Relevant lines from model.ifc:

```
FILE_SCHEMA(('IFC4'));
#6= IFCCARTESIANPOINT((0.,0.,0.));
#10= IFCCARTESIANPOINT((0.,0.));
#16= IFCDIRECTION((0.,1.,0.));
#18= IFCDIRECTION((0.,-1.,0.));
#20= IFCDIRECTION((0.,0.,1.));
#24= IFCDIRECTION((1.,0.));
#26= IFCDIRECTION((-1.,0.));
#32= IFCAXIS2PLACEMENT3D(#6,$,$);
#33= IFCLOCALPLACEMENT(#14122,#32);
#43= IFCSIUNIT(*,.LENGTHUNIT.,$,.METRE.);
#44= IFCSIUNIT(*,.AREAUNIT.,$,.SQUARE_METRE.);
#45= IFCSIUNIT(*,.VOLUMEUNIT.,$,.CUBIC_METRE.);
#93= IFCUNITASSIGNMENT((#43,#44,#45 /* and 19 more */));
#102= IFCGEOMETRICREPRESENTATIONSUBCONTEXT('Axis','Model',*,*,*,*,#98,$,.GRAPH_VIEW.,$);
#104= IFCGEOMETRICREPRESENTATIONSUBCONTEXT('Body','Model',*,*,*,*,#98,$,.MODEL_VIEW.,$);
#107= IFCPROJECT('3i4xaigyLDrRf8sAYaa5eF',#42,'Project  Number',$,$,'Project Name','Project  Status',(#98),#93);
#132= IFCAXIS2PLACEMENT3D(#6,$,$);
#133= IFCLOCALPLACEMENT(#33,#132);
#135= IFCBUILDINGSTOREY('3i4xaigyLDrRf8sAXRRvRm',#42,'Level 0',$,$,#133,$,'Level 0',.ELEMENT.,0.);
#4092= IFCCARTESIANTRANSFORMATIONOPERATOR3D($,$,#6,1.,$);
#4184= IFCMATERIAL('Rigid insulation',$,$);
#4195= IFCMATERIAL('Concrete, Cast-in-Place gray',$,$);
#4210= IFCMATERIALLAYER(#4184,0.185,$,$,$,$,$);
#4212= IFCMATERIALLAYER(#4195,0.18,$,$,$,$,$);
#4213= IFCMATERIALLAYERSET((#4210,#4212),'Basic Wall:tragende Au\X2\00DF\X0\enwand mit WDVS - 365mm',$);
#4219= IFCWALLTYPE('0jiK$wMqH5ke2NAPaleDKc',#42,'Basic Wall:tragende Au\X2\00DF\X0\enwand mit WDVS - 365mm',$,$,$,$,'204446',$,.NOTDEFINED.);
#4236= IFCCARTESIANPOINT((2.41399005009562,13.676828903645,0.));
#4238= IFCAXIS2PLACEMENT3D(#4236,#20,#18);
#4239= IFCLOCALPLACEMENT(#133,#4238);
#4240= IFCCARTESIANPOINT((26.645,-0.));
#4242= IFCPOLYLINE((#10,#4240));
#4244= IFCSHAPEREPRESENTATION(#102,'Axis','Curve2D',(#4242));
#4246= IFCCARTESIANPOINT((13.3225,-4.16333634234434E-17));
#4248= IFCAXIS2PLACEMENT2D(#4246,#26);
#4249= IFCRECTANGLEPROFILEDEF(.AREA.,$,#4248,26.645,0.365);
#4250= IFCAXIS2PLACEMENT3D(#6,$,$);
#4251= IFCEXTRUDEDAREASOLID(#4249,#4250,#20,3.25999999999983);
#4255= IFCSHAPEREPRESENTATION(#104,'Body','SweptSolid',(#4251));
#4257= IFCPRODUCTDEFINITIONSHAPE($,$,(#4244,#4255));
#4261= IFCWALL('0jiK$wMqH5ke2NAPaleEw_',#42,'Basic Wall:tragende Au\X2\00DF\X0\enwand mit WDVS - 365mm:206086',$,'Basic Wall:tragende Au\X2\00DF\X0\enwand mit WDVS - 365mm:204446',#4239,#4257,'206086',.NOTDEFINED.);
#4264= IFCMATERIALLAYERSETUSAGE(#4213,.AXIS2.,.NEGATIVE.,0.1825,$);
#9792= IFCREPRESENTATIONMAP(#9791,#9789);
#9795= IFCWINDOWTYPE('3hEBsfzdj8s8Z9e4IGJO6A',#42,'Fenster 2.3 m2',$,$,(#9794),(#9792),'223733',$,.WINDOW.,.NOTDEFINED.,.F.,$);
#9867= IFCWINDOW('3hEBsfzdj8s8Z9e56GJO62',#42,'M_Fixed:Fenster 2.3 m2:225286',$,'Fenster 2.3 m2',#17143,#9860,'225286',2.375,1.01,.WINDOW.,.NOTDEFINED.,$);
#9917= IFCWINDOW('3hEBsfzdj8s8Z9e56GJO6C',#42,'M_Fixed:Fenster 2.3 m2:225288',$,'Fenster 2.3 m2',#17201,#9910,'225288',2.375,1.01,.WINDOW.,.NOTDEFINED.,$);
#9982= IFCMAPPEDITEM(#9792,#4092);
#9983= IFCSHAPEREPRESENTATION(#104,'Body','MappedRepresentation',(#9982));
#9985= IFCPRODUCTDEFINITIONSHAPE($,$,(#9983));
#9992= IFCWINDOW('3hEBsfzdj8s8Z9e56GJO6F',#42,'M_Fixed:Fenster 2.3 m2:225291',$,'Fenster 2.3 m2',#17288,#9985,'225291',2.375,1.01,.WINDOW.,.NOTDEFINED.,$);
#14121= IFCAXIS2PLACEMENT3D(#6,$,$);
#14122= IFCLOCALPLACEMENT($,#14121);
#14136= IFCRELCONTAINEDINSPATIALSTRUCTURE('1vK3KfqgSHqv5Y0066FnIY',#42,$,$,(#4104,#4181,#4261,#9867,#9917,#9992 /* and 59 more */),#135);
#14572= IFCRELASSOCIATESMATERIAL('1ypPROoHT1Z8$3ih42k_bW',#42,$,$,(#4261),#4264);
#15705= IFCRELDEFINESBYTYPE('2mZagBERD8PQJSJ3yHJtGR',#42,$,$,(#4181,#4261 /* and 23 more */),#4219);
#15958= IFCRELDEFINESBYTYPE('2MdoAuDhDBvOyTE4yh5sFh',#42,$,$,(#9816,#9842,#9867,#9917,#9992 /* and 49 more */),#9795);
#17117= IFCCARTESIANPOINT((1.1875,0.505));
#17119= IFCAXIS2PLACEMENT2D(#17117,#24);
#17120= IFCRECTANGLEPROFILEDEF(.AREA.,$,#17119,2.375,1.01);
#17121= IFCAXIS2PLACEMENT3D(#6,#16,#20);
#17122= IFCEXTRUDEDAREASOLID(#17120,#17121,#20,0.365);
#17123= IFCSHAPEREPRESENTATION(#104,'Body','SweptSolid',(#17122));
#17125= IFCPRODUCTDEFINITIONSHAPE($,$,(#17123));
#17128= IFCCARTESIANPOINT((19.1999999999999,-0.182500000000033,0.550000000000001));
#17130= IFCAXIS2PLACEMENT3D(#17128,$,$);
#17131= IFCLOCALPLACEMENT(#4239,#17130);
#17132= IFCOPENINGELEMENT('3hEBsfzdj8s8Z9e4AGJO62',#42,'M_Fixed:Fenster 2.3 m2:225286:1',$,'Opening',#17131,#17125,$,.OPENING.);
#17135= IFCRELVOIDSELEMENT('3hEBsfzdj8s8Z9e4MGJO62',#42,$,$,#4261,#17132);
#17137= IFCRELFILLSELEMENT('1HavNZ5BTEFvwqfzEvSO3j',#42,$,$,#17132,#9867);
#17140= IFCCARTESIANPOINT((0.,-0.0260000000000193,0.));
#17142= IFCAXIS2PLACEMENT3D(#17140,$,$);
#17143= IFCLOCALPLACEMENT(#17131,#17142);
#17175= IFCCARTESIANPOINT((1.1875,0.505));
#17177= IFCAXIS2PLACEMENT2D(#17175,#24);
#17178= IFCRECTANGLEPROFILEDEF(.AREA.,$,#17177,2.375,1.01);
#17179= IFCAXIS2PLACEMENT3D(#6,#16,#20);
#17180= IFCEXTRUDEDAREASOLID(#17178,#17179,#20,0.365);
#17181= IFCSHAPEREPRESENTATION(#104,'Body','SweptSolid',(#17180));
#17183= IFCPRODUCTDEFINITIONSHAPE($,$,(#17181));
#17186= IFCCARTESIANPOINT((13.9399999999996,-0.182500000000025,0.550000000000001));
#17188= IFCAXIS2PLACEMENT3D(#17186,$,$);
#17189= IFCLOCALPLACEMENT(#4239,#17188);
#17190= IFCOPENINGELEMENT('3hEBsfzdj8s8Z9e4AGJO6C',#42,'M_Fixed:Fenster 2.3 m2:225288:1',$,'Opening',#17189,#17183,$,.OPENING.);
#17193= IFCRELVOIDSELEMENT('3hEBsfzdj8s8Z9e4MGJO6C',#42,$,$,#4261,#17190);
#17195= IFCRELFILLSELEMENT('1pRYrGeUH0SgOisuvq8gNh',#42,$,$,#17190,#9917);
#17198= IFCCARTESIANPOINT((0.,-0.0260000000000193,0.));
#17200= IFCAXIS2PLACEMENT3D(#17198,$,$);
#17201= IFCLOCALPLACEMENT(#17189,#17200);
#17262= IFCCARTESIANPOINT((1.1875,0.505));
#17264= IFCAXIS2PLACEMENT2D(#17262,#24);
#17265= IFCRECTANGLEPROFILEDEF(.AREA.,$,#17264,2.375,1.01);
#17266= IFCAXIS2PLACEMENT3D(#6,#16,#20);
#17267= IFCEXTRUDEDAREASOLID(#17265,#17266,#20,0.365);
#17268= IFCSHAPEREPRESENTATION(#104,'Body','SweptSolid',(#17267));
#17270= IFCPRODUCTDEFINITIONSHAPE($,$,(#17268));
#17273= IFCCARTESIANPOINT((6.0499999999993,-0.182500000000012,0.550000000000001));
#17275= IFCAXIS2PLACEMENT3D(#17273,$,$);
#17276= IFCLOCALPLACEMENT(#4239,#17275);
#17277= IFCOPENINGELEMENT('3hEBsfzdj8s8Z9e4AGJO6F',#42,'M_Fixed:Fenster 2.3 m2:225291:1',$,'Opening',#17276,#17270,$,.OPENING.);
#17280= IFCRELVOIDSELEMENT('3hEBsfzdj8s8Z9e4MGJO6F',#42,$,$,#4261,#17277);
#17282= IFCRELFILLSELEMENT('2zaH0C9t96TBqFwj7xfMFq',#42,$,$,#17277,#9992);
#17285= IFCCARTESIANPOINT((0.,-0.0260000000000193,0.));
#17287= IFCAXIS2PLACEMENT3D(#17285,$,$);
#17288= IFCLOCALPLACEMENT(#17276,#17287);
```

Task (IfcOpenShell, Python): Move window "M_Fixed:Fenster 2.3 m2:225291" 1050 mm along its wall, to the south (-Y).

```python
import ifcopenshell
import ifcopenshell.api.geometry
import ifcopenshell.util.placement
import ifcopenshell.util.unit

model = ifcopenshell.open("model.ifc")
unit_scale = ifcopenshell.util.unit.calculate_unit_scale(model)

window = model.by_id(9992)
opening = window.FillsVoids[0].RelatingOpeningElement
wall = opening.VoidsElements[0].RelatingBuildingElement

wall_matrix = ifcopenshell.util.placement.get_local_placement(wall.ObjectPlacement)
shift = wall_matrix[:3, 0] * 1.05 / unit_scale
before = ifcopenshell.util.placement.get_local_placement(window.ObjectPlacement)[:3, 3].copy()

# The window is placed relative to its opening, so it follows when the opening moves.
matrix = ifcopenshell.util.placement.get_local_placement(opening.ObjectPlacement)
matrix[:3, 3] += shift
ifcopenshell.api.geometry.edit_object_placement(
    model, product=opening, matrix=matrix, is_si=False, should_transform_children=True
)

after = ifcopenshell.util.placement.get_local_placement(window.ObjectPlacement)[:3, 3]
print("window moved by", (after - before).round(3) + 0.0)

model.write("model_v2.ifc")
```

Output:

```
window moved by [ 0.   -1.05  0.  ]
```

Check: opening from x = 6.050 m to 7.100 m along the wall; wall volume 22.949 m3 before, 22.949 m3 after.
